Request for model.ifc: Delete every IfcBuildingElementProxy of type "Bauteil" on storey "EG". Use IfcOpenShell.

First a look at what the model holds.

```python
import ifcopenshell
import ifcopenshell.util.element

model = ifcopenshell.open("model.ifc")
print(model.schema)
storey = next(s for s in model.by_type("IfcBuildingStorey") if s.Name == "EG")
proxies = [e for e in ifcopenshell.util.element.get_decomposition(storey) if e.is_a("IfcBuildingElementProxy")]
seen = {}
for e in proxies:
    element_type = ifcopenshell.util.element.get_type(e)
    name = element_type.Name if element_type not in (None, e) else None
    seen[name] = seen.get(name, 0) + 1
for name, count in sorted(seen.items(), key=str):
    print(count, "x", name)
```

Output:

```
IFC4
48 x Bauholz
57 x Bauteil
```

```python
import ifcopenshell
import ifcopenshell.api.root
import ifcopenshell.util.element

model = ifcopenshell.open("model.ifc")

storey = next(s for s in model.by_type("IfcBuildingStorey") if s.Name == "EG")
proxies = [e for e in ifcopenshell.util.element.get_decomposition(storey) if e.is_a("IfcBuildingElementProxy")]
targets = [e for e in proxies if (t := ifcopenshell.util.element.get_type(e)) not in (None, e) and t.Name == "Bauteil"]

for e in targets:
    ifcopenshell.api.root.remove_product(model, product=e)
print(len(targets), "removed")

model.write("model_v2.ifc")
```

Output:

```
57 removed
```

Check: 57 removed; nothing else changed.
